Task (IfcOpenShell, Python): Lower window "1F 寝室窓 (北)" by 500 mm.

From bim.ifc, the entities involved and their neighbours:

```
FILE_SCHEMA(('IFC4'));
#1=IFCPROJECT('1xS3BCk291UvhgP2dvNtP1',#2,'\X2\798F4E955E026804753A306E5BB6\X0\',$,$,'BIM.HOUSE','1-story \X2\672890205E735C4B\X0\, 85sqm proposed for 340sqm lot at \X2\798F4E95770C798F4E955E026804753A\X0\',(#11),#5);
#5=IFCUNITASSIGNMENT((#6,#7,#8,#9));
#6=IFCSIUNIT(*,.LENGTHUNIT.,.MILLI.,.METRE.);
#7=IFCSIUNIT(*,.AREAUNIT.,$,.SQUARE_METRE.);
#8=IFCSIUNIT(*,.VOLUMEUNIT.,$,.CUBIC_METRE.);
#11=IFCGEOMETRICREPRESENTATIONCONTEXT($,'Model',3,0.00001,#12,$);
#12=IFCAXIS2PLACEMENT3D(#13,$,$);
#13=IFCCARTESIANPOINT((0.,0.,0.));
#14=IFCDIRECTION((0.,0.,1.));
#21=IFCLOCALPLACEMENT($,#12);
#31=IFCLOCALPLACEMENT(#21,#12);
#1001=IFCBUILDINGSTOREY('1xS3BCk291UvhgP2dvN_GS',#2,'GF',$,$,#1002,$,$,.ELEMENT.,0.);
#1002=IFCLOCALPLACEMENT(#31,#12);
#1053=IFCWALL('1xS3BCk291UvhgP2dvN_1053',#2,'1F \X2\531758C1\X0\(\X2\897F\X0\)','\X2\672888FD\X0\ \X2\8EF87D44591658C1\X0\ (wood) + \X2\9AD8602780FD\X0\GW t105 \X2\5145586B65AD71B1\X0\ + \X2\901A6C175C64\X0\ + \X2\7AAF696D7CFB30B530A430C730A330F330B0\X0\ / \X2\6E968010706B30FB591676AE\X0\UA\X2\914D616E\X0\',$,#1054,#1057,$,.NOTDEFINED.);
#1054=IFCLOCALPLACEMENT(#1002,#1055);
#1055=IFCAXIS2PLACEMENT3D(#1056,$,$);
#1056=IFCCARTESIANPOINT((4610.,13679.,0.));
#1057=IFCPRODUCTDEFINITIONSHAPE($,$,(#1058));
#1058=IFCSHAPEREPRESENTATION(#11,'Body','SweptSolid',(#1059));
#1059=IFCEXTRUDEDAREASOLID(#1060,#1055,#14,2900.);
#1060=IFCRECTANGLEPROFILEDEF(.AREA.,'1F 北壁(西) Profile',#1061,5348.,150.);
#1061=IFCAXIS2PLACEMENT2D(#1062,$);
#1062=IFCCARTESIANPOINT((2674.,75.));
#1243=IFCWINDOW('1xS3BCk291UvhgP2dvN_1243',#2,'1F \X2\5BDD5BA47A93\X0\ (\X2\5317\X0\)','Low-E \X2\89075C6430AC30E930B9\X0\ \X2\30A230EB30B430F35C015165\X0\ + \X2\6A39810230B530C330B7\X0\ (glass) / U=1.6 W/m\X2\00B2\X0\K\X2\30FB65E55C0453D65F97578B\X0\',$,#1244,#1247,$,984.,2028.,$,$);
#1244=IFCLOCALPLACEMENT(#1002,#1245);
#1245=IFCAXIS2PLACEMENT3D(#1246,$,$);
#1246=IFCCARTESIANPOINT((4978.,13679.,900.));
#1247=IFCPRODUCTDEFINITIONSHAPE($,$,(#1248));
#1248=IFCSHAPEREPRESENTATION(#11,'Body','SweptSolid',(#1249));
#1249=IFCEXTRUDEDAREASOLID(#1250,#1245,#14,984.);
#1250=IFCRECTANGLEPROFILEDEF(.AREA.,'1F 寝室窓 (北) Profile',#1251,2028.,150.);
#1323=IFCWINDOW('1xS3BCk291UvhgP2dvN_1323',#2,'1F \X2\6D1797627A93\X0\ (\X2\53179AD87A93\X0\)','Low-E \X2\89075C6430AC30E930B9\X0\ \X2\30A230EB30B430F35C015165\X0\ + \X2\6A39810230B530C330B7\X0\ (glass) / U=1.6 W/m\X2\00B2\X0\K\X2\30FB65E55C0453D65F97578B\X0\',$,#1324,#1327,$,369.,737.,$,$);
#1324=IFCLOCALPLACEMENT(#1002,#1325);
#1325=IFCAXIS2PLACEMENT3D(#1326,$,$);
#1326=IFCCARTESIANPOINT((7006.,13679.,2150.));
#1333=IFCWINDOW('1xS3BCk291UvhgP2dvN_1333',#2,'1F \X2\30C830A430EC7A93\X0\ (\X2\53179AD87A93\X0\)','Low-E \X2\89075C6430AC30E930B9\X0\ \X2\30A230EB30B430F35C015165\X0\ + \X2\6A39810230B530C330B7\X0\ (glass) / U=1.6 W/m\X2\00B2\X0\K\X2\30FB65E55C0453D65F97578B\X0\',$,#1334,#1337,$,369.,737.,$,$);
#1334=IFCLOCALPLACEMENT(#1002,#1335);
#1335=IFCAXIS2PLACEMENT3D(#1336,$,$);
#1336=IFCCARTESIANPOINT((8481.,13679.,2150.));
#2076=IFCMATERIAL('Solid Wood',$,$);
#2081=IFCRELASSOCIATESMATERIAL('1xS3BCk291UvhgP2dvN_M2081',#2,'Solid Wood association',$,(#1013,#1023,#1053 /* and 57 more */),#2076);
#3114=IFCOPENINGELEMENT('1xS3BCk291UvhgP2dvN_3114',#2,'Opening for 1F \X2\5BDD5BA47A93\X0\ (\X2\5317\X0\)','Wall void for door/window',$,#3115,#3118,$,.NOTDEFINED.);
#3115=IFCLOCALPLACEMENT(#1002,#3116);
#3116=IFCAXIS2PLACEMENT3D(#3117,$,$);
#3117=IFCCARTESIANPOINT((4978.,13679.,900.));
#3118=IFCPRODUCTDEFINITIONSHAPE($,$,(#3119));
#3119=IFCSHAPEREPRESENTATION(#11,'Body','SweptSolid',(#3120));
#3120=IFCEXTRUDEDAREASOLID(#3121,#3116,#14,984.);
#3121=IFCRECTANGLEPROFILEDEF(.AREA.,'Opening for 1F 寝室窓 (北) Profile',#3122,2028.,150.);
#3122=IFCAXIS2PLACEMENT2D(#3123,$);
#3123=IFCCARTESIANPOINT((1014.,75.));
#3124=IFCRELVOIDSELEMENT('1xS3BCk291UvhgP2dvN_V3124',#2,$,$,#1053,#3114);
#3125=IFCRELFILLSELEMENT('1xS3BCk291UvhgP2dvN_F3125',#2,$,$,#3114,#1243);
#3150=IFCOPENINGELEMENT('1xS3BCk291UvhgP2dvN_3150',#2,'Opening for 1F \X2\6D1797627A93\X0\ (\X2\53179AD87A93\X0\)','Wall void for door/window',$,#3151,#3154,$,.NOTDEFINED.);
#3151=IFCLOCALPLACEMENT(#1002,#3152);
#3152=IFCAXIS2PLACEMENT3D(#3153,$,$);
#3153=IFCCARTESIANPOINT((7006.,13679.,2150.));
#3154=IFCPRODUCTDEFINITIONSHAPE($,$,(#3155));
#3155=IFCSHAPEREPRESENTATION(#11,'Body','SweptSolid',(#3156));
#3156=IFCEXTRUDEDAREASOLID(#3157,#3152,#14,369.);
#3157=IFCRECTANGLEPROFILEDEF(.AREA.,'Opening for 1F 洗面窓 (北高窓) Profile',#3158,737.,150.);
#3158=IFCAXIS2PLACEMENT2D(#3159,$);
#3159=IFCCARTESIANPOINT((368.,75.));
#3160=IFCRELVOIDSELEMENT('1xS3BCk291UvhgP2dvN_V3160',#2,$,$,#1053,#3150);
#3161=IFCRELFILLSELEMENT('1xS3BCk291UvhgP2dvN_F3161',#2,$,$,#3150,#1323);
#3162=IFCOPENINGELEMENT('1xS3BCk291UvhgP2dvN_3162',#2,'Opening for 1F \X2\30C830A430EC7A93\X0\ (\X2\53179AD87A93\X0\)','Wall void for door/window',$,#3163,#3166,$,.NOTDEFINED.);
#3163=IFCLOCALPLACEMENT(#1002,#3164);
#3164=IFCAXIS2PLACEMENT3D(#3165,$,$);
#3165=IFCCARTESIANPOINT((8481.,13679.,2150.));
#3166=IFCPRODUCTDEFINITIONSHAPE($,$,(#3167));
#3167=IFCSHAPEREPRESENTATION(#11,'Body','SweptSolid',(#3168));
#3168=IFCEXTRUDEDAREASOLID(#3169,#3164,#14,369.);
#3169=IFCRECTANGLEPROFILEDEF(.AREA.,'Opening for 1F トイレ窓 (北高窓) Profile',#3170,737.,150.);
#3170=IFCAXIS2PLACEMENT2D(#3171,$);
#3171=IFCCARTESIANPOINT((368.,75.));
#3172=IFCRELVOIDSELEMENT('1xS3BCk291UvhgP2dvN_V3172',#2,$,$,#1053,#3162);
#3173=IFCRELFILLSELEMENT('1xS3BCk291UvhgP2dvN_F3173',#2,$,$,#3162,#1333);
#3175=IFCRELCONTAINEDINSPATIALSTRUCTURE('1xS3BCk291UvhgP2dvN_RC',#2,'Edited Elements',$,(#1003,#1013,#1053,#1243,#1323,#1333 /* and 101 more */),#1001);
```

```python
import numpy as np
import ifcopenshell
import ifcopenshell.api.geometry
import ifcopenshell.util.placement
import ifcopenshell.util.unit

model = ifcopenshell.open("bim.ifc")
unit_scale = ifcopenshell.util.unit.calculate_unit_scale(model)

window = model.by_guid("1xS3BCk291UvhgP2dvN_1243")
opening = window.FillsVoids[0].RelatingOpeningElement
dz = -0.5 / unit_scale

shift = np.array([0.0, 0.0, dz])
# The window is not placed relative to its opening, so move both.
for product in (opening, window):
    matrix = ifcopenshell.util.placement.get_local_placement(product.ObjectPlacement)
    matrix[:3, 3] += shift
    ifcopenshell.api.geometry.edit_object_placement(model, product=product, matrix=matrix, is_si=False)

print(f"moved by {dz * unit_scale:+.3f} m")

model.write("bim_v2.ifc")
```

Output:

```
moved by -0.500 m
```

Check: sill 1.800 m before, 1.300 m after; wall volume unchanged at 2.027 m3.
